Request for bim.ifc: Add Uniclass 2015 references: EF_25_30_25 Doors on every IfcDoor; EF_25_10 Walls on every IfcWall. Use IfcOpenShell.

First a look at what the model holds.

```python
import ifcopenshell

model = ifcopenshell.open("bim.ifc")
print(model.schema)
print("classifications:", [c.Name for c in model.by_type("IfcClassification")])
for ifc_class in ("IfcDoor", "IfcRoof", "IfcStair", "IfcWall", "IfcWindow"):
    print(ifc_class, len(model.by_type(ifc_class)))
```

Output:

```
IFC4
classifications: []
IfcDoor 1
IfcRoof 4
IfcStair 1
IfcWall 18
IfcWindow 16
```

```python
import ifcopenshell
import ifcopenshell.api.classification

model = ifcopenshell.open("bim.ifc")

system = ifcopenshell.api.classification.add_classification(model, classification="Uniclass 2015")

codes = {
    "IfcDoor": ("EF_25_30_25", "Doors"),
    "IfcWall": ("EF_25_10", "Walls"),
}
for ifc_class, (code, name) in codes.items():
    products = model.by_type(ifc_class)
    ifcopenshell.api.classification.add_reference(
        model, products=products, classification=system, identification=code, name=name
    )
    print(code, len(products))

model.write("bim_edited.ifc")
```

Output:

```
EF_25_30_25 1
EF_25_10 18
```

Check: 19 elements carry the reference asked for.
